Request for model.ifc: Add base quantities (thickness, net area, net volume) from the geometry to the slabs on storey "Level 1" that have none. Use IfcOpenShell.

First a look at what the model holds.

```python
import ifcopenshell
import ifcopenshell.util.element
import ifcopenshell.util.unit

model = ifcopenshell.open("model.ifc")
print(model.schema)
for unit_type in ("LENGTHUNIT", "AREAUNIT", "VOLUMEUNIT"):
    print(unit_type, ifcopenshell.util.unit.calculate_unit_scale(model, unit_type))
storey = next(s for s in model.by_type("IfcBuildingStorey") if s.Name == "Level 1")
slabs = [e for e in ifcopenshell.util.element.get_decomposition(storey) if e.is_a("IfcSlab")]
for e in sorted(slabs, key=lambda e: e.id()):
    print(e.id(), e.is_a(), e.Name, list(ifcopenshell.util.element.get_psets(e, qtos_only=True)), sep=" | ")
```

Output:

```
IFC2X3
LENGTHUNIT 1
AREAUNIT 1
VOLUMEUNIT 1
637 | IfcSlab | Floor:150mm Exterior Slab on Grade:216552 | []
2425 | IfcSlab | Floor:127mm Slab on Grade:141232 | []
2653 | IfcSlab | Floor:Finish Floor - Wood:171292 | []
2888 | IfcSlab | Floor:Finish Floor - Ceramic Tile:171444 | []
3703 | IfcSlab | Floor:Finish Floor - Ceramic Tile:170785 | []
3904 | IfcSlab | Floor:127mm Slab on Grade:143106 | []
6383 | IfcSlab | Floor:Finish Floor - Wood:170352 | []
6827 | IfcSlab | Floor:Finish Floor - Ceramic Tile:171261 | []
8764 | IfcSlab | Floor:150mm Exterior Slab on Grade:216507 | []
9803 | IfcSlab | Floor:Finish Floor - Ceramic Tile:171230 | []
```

```python
import ifcopenshell
import ifcopenshell.api.pset
import ifcopenshell.geom
import ifcopenshell.util.element
import ifcopenshell.util.shape
import ifcopenshell.util.unit

model = ifcopenshell.open("model.ifc")
unit_scale = ifcopenshell.util.unit.calculate_unit_scale(model)
area_scale = ifcopenshell.util.unit.calculate_unit_scale(model, "AREAUNIT")
volume_scale = ifcopenshell.util.unit.calculate_unit_scale(model, "VOLUMEUNIT")
settings = ifcopenshell.geom.settings()

storey = next(s for s in model.by_type("IfcBuildingStorey") if s.Name == "Level 1")
slabs = [e for e in ifcopenshell.util.element.get_decomposition(storey) if e.is_a("IfcSlab")]

for e in sorted(slabs, key=lambda e: e.id()):
    if ifcopenshell.util.element.get_psets(e, qtos_only=True, should_inherit=False):
        continue
    # Geometry comes back in metres, in the element's own axes.
    shape = ifcopenshell.geom.create_shape(settings, e)
    values = {
        "Width": ifcopenshell.util.shape.get_z(shape.geometry) / unit_scale,
        "NetArea": ifcopenshell.util.shape.get_footprint_area(shape.geometry) / area_scale,
        "NetVolume": ifcopenshell.util.shape.get_volume(shape.geometry) / volume_scale,
    }
    qto = ifcopenshell.api.pset.add_qto(model, product=e, name="BaseQuantities")
    ifcopenshell.api.pset.edit_qto(model, qto=qto, properties=values)
    print(e.id(), {k: round(v, 3) for k, v in values.items()})

model.write("model_v2.ifc")
```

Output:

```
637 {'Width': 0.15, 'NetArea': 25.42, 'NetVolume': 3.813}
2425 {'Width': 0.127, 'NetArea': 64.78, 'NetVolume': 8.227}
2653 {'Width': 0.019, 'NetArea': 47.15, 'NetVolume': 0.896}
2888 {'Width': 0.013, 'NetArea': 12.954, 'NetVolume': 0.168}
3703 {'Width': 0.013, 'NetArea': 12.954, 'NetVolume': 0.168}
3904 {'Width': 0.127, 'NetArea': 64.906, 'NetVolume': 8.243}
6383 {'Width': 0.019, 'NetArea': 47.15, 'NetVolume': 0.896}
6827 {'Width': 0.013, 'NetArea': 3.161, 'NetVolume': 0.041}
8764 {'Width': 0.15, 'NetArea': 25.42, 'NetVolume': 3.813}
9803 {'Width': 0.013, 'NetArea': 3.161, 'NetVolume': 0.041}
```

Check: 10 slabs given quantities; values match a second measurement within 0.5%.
